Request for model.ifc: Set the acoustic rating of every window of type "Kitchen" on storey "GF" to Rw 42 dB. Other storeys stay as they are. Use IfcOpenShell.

First a look at what the model holds.

```python
import ifcopenshell
import ifcopenshell.util.element

model = ifcopenshell.open("model.ifc")
print(model.schema)
storey = next(s for s in model.by_type("IfcBuildingStorey") if s.Name == "GF")
windows = [e for e in ifcopenshell.util.element.get_decomposition(storey) if e.is_a("IfcWindow")]
seen = {}
for e in windows:
    element_type = ifcopenshell.util.element.get_type(e)
    key = (element_type.Name if element_type != e and element_type else None, ifcopenshell.util.element.get_pset(e, "Pset_WindowCommon", "AcousticRating"))
    seen[key] = seen.get(key, 0) + 1
for (name, value), count in sorted(seen.items(), key=str):
    print(count, "x", name, "|", value)
```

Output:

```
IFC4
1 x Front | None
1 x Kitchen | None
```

```python
import ifcopenshell
import ifcopenshell.api.pset
import ifcopenshell.util.element

model = ifcopenshell.open("model.ifc")

storey = next(s for s in model.by_type("IfcBuildingStorey") if s.Name == "GF")
windows = [e for e in ifcopenshell.util.element.get_decomposition(storey) if e.is_a("IfcWindow")]

count = 0
for e in windows:
    element_type = ifcopenshell.util.element.get_type(e)
    if element_type in (None, e) or element_type.Name != "Kitchen":
        continue
    # add_pset returns the element's existing set when there is one.
    pset = ifcopenshell.api.pset.add_pset(model, product=e, name="Pset_WindowCommon")
    ifcopenshell.api.pset.edit_pset(model, pset=pset, properties={"AcousticRating": "Rw 42 dB"})
    count += 1

print(count, "windows updated")

model.write("model_updated.ifc")
```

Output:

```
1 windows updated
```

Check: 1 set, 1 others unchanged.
